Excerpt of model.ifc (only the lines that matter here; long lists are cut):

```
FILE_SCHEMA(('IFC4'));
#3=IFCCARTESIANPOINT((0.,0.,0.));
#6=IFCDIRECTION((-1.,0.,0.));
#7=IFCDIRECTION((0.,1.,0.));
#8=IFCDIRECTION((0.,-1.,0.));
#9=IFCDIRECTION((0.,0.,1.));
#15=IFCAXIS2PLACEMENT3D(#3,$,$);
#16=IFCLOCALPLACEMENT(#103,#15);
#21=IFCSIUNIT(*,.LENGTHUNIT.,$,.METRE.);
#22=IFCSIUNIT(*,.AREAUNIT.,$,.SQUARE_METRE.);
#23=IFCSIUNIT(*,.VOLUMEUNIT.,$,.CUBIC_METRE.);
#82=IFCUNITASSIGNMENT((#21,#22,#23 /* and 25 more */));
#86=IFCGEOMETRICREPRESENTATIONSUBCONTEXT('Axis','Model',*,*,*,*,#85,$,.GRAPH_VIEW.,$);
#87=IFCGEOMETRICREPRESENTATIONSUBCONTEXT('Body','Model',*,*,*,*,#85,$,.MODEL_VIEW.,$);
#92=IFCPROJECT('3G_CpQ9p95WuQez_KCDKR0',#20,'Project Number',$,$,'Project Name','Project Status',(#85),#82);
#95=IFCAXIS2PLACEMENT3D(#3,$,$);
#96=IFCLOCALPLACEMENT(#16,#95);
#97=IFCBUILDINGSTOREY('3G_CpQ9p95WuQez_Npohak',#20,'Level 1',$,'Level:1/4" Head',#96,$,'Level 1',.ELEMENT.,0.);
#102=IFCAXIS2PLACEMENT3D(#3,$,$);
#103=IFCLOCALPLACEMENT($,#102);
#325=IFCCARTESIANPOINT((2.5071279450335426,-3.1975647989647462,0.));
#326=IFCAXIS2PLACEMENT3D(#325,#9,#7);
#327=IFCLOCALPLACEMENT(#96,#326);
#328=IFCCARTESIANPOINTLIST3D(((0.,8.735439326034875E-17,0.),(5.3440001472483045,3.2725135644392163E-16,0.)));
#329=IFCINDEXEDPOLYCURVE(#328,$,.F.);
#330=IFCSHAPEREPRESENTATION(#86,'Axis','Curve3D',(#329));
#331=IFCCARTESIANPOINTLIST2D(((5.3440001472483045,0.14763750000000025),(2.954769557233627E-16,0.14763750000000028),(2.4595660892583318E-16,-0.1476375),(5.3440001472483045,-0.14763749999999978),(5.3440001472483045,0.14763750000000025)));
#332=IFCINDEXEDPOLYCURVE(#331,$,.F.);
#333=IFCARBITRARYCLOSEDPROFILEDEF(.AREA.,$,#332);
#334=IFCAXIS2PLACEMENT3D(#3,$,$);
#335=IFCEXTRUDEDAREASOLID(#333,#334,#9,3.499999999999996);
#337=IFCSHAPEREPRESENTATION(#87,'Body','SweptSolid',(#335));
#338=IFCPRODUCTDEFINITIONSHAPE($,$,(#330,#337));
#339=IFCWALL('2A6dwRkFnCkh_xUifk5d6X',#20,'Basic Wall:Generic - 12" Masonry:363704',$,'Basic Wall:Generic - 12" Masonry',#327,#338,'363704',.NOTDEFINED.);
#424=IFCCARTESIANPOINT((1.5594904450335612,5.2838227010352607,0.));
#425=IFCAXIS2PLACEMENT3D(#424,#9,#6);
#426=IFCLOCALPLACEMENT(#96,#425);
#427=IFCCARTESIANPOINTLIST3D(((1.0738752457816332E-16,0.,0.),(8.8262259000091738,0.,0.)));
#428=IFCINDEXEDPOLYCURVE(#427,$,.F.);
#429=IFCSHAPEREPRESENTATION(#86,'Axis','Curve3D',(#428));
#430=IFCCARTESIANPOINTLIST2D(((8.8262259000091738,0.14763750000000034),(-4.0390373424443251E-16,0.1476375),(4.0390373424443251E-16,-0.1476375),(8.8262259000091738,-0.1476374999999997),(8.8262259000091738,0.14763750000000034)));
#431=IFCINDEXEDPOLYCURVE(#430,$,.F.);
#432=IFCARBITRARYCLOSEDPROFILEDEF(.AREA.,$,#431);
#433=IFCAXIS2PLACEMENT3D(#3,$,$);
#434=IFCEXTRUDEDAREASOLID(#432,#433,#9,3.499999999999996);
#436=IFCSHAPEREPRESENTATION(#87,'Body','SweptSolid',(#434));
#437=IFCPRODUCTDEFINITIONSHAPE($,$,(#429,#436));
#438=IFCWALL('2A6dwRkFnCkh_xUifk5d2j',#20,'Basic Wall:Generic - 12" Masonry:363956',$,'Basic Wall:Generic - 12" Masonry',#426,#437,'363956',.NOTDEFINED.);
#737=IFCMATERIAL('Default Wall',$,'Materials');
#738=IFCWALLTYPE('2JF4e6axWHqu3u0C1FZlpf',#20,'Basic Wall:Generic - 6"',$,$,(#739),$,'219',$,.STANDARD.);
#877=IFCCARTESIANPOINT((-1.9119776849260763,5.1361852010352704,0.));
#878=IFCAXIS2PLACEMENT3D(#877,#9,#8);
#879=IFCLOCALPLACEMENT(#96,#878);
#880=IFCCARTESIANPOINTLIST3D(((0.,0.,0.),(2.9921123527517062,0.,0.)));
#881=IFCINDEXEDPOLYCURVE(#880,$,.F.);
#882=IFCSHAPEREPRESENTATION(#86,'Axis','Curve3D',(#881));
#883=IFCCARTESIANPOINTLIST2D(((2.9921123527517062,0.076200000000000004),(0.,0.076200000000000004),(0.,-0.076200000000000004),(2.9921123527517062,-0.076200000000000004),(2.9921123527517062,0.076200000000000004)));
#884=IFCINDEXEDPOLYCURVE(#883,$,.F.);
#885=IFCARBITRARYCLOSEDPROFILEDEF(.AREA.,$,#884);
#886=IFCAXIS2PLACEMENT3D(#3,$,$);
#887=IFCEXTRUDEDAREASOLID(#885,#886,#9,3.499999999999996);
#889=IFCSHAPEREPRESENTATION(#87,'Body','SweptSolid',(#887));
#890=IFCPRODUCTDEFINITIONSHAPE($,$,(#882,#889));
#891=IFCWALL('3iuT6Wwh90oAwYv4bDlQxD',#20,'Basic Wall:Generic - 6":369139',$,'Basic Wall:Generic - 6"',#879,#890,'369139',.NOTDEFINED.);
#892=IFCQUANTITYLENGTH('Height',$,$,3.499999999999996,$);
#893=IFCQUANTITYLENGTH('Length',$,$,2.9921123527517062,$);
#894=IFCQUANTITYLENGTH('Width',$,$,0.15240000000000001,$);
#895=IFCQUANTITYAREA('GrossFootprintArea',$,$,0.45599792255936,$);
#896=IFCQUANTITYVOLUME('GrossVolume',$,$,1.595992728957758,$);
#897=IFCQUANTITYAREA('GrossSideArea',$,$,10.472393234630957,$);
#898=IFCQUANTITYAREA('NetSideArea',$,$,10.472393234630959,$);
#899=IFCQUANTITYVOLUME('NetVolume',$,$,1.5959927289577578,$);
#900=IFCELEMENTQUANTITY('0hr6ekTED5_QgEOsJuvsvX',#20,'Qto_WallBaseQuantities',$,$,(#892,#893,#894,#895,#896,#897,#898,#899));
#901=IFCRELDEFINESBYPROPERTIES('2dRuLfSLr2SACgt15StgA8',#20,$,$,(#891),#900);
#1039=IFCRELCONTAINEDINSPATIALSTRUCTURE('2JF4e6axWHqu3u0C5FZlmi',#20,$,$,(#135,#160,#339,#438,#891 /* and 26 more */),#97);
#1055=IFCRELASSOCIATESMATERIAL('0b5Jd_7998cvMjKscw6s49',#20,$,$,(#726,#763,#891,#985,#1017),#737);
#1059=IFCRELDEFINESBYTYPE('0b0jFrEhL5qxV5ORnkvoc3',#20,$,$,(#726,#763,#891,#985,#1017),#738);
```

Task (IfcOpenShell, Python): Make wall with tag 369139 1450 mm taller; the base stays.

```python
import ifcopenshell
import ifcopenshell.api.pset
import ifcopenshell.geom
import ifcopenshell.util.element
import ifcopenshell.util.representation
import ifcopenshell.util.shape
import ifcopenshell.util.unit

model = ifcopenshell.open("model.ifc")
unit_scale = ifcopenshell.util.unit.calculate_unit_scale(model)
area_scale = ifcopenshell.util.unit.calculate_unit_scale(model, "AREAUNIT")
volume_scale = ifcopenshell.util.unit.calculate_unit_scale(model, "VOLUMEUNIT")
settings = ifcopenshell.geom.settings()


def volume(element):
    """Net volume in cubic metres, openings subtracted."""
    shape = ifcopenshell.geom.create_shape(settings, element)
    return ifcopenshell.util.shape.get_volume(shape.geometry)


wall = model.by_guid("3iuT6Wwh90oAwYv4bDlQxD")
before = volume(wall)

body = ifcopenshell.util.representation.get_representation(wall, "Model", "Body")
solid = body.Items[0]
old_height = solid.Depth
solid.Depth += 1.45 / unit_scale
after = volume(wall)
thickness = 0.1524  # wall thickness in metres

# Update the stored height, areas and volumes.
qto = model.by_id(ifcopenshell.util.element.get_pset(wall, "Qto_WallBaseQuantities", should_inherit=False)["id"])
ifcopenshell.api.pset.edit_qto(model, qto=qto, properties={
    "Height": solid.Depth,
    "GrossVolume": ifcopenshell.util.element.get_pset(wall, "Qto_WallBaseQuantities", "GrossVolume") * solid.Depth / old_height,
    "GrossSideArea": ifcopenshell.util.element.get_pset(wall, "Qto_WallBaseQuantities", "GrossSideArea") * solid.Depth / old_height,
    "NetSideArea": after / thickness / area_scale,
    "NetVolume": after / volume_scale,
})

print(f"height {old_height:g} -> {solid.Depth:g}, volume {before:.3f} -> {after:.3f} m3")

model.write("model_updated.ifc")
```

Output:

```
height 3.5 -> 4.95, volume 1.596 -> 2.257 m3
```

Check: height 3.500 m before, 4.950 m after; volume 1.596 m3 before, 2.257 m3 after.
